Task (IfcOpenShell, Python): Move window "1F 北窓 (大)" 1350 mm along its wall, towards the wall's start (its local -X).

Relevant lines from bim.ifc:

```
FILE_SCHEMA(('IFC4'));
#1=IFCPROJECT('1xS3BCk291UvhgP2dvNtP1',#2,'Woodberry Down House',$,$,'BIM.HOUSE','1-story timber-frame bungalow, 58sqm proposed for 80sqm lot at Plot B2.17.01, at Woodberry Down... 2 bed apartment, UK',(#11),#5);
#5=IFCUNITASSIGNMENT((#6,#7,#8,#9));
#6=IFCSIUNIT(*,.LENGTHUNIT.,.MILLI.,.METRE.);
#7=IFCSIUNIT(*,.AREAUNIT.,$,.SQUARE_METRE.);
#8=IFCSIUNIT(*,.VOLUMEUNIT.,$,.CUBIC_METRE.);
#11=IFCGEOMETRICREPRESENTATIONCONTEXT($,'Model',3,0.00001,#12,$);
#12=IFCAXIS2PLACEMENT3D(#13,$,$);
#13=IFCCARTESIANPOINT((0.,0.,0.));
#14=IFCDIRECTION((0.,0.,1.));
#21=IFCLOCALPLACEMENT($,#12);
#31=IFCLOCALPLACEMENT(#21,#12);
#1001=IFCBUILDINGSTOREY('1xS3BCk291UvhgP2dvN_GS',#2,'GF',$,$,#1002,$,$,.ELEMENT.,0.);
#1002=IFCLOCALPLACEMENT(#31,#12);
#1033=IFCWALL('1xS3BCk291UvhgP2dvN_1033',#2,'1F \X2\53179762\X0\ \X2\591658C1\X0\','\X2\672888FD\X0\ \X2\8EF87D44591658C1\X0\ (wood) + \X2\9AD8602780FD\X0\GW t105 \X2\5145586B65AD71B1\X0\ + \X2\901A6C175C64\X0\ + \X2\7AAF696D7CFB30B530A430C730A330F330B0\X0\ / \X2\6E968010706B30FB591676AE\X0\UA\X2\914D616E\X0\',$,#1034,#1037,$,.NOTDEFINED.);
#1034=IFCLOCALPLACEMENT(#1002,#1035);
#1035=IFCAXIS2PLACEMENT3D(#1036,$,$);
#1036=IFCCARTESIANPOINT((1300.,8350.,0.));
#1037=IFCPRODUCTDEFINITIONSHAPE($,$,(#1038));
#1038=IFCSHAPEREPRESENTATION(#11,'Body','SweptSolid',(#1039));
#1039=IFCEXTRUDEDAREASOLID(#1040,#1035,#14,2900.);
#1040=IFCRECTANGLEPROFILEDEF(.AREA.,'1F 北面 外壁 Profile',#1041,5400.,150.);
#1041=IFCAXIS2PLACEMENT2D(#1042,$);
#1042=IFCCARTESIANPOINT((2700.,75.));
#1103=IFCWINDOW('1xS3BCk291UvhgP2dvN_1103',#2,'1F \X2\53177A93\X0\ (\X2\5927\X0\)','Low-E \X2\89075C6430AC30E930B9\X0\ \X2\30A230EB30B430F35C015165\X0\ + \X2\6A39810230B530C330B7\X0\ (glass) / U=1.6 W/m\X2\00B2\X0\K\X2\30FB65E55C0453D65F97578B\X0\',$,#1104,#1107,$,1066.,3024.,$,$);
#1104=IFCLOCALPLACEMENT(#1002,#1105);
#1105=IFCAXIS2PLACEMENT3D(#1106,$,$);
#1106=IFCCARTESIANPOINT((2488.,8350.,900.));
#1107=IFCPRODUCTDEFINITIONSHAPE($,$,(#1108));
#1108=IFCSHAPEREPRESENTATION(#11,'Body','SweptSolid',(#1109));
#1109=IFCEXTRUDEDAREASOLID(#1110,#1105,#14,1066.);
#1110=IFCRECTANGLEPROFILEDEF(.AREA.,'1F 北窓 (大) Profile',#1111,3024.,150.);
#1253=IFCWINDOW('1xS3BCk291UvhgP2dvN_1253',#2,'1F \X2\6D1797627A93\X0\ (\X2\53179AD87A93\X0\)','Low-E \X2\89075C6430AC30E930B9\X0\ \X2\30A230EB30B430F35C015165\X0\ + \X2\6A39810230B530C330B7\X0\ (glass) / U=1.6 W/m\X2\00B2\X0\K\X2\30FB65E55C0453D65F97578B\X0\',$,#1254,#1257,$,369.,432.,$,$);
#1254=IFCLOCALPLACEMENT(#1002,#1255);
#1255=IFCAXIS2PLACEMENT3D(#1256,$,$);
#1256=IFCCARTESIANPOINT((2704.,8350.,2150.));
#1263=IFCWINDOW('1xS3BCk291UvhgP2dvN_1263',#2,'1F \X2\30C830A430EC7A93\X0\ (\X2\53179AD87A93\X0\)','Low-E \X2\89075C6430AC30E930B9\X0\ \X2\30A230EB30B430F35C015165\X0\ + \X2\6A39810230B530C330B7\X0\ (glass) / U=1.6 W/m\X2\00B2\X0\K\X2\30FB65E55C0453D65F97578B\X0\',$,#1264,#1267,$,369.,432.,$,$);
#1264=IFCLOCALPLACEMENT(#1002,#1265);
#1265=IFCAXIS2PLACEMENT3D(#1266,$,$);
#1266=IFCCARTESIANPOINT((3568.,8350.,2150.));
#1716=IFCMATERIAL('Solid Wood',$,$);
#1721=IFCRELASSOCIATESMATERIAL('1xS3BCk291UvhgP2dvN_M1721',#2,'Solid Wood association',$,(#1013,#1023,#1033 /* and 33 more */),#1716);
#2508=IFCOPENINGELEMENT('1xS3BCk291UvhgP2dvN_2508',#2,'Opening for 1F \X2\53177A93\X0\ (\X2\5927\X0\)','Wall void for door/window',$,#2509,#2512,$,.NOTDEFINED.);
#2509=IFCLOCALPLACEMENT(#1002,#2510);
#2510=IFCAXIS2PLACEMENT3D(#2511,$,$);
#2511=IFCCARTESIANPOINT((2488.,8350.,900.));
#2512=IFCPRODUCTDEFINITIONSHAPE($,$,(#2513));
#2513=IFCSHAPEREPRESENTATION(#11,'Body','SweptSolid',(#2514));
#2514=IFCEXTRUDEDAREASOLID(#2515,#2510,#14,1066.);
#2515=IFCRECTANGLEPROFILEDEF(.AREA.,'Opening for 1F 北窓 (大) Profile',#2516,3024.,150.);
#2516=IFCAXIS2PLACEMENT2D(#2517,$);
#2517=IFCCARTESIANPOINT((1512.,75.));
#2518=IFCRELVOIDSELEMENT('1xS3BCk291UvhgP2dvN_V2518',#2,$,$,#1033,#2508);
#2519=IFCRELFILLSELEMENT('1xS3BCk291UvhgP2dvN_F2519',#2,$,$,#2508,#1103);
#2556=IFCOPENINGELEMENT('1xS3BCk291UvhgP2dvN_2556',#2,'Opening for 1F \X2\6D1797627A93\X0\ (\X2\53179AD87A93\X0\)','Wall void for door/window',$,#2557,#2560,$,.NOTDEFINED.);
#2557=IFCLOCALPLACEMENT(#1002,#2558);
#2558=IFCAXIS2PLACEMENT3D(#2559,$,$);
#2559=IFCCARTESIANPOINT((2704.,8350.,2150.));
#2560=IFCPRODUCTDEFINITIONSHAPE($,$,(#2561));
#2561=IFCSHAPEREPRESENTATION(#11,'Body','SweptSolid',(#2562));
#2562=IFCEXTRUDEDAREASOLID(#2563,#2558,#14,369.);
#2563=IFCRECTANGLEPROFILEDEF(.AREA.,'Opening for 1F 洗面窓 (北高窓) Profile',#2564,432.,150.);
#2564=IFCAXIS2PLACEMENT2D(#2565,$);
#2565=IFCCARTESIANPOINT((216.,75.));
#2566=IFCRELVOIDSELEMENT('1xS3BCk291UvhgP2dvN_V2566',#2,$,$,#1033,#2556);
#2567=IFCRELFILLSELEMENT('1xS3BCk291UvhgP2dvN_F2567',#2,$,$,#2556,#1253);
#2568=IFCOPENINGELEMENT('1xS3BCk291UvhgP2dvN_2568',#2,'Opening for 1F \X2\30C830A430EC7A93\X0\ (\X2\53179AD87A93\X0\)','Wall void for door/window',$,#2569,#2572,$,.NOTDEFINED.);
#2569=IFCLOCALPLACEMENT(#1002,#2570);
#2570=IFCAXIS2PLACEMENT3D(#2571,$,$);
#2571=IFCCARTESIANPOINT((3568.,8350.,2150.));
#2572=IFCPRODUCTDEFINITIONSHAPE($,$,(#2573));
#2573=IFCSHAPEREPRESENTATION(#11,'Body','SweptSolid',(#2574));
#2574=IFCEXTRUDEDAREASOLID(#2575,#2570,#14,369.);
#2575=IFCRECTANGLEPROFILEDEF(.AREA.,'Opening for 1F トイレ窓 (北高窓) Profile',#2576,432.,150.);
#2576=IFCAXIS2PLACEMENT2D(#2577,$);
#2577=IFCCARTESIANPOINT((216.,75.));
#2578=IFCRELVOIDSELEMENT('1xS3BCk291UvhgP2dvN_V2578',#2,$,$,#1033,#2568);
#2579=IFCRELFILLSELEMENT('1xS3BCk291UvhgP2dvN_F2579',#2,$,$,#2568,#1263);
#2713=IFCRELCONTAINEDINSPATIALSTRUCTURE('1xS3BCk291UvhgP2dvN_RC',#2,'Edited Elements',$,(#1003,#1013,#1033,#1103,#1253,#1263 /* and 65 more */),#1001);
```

```python
import ifcopenshell
import ifcopenshell.api.geometry
import ifcopenshell.util.placement
import ifcopenshell.util.unit

model = ifcopenshell.open("bim.ifc")
unit_scale = ifcopenshell.util.unit.calculate_unit_scale(model)

window = model.by_guid("1xS3BCk291UvhgP2dvN_1103")
opening = window.FillsVoids[0].RelatingOpeningElement
wall = opening.VoidsElements[0].RelatingBuildingElement

wall_matrix = ifcopenshell.util.placement.get_local_placement(wall.ObjectPlacement)
shift = wall_matrix[:3, 0] * -1.35 / unit_scale
before = ifcopenshell.util.placement.get_local_placement(window.ObjectPlacement)[:3, 3].copy()

# The window is not placed relative to its opening, so move both.
for product in (opening, window):
    matrix = ifcopenshell.util.placement.get_local_placement(product.ObjectPlacement)
    matrix[:3, 3] += shift
    ifcopenshell.api.geometry.edit_object_placement(model, product=product, matrix=matrix, is_si=False)

after = ifcopenshell.util.placement.get_local_placement(window.ObjectPlacement)[:3, 3]
print("window moved by", (after - before).round(3) + 0.0)

model.write("bim_rev.ifc")
```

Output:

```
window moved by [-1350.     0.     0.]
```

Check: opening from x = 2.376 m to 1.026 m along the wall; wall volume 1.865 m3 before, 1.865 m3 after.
